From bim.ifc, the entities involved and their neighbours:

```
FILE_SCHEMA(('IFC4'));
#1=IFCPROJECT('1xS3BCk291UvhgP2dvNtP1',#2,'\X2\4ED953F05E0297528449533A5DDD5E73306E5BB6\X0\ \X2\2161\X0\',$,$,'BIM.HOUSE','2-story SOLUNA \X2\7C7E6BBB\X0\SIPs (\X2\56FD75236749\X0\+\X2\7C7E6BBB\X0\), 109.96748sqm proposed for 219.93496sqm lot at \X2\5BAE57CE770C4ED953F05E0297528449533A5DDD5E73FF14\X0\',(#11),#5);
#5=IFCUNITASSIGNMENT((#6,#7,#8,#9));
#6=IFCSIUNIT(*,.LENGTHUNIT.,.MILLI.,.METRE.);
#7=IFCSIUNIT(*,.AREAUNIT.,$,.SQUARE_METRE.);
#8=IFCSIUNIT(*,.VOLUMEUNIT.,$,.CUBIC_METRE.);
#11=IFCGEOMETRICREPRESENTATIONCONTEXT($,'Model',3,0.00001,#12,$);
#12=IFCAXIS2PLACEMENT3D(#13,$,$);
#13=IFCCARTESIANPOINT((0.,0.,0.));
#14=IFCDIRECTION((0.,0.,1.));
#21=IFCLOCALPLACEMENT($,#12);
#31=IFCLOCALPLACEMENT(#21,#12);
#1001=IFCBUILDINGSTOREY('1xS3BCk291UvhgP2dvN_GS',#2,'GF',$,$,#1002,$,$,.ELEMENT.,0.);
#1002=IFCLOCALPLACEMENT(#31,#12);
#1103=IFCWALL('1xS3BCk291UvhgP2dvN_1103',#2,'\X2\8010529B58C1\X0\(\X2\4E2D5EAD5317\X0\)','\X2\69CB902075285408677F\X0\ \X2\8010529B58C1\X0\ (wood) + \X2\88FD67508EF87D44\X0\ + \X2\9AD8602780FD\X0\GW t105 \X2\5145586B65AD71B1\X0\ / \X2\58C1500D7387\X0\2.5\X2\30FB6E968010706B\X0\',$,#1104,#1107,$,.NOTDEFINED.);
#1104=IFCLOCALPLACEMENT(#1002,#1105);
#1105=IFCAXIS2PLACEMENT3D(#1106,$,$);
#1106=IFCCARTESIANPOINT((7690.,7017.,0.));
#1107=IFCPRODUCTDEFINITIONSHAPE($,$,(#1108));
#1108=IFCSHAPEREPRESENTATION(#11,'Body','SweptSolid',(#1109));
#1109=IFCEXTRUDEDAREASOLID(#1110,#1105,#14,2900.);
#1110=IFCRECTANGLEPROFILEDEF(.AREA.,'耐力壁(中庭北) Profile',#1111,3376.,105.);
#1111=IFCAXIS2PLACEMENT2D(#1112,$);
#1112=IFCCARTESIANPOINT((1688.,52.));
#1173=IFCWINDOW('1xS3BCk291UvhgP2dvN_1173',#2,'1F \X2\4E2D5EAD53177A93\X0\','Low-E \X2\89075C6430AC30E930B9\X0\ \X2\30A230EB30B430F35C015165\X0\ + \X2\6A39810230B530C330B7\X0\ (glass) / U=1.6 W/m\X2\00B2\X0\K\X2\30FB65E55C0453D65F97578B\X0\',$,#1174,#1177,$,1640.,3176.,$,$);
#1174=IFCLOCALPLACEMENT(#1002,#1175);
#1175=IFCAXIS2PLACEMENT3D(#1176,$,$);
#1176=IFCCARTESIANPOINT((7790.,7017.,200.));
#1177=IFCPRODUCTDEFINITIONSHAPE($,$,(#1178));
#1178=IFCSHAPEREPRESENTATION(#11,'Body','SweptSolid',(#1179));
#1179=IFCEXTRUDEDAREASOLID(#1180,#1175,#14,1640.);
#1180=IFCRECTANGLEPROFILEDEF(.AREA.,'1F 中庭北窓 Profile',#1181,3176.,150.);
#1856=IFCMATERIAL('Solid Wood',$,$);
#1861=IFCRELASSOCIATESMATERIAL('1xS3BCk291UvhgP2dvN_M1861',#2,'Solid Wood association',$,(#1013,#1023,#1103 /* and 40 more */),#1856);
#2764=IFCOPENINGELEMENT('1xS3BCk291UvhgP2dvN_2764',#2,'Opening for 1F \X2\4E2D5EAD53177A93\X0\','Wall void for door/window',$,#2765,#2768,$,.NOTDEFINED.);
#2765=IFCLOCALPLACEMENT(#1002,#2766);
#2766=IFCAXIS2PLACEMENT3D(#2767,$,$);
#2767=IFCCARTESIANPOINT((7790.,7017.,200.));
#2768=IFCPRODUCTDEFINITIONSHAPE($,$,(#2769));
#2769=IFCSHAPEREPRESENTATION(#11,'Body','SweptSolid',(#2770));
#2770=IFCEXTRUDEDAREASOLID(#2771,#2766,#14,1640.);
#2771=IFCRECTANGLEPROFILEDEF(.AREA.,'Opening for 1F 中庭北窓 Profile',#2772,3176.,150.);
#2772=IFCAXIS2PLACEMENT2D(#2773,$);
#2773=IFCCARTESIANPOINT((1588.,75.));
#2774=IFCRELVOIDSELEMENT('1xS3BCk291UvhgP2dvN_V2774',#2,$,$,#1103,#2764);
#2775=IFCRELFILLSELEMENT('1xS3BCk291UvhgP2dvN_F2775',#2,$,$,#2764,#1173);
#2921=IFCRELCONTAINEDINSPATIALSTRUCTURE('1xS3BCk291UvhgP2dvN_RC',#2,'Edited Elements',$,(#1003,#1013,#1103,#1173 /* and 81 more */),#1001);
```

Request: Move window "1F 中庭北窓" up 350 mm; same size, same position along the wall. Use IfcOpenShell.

```python
import numpy as np
import ifcopenshell
import ifcopenshell.api.geometry
import ifcopenshell.util.placement
import ifcopenshell.util.unit

model = ifcopenshell.open("bim.ifc")
unit_scale = ifcopenshell.util.unit.calculate_unit_scale(model)

window = model.by_id(1173)
opening = window.FillsVoids[0].RelatingOpeningElement
dz = 0.35 / unit_scale

shift = np.array([0.0, 0.0, dz])
# The window is not placed relative to its opening, so move both.
for product in (opening, window):
    matrix = ifcopenshell.util.placement.get_local_placement(product.ObjectPlacement)
    matrix[:3, 3] += shift
    ifcopenshell.api.geometry.edit_object_placement(model, product=product, matrix=matrix, is_si=False)

print(f"moved by {dz * unit_scale:+.3f} m")

model.write("bim-out.ifc")
```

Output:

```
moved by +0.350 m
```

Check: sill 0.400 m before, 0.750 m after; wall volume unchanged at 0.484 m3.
